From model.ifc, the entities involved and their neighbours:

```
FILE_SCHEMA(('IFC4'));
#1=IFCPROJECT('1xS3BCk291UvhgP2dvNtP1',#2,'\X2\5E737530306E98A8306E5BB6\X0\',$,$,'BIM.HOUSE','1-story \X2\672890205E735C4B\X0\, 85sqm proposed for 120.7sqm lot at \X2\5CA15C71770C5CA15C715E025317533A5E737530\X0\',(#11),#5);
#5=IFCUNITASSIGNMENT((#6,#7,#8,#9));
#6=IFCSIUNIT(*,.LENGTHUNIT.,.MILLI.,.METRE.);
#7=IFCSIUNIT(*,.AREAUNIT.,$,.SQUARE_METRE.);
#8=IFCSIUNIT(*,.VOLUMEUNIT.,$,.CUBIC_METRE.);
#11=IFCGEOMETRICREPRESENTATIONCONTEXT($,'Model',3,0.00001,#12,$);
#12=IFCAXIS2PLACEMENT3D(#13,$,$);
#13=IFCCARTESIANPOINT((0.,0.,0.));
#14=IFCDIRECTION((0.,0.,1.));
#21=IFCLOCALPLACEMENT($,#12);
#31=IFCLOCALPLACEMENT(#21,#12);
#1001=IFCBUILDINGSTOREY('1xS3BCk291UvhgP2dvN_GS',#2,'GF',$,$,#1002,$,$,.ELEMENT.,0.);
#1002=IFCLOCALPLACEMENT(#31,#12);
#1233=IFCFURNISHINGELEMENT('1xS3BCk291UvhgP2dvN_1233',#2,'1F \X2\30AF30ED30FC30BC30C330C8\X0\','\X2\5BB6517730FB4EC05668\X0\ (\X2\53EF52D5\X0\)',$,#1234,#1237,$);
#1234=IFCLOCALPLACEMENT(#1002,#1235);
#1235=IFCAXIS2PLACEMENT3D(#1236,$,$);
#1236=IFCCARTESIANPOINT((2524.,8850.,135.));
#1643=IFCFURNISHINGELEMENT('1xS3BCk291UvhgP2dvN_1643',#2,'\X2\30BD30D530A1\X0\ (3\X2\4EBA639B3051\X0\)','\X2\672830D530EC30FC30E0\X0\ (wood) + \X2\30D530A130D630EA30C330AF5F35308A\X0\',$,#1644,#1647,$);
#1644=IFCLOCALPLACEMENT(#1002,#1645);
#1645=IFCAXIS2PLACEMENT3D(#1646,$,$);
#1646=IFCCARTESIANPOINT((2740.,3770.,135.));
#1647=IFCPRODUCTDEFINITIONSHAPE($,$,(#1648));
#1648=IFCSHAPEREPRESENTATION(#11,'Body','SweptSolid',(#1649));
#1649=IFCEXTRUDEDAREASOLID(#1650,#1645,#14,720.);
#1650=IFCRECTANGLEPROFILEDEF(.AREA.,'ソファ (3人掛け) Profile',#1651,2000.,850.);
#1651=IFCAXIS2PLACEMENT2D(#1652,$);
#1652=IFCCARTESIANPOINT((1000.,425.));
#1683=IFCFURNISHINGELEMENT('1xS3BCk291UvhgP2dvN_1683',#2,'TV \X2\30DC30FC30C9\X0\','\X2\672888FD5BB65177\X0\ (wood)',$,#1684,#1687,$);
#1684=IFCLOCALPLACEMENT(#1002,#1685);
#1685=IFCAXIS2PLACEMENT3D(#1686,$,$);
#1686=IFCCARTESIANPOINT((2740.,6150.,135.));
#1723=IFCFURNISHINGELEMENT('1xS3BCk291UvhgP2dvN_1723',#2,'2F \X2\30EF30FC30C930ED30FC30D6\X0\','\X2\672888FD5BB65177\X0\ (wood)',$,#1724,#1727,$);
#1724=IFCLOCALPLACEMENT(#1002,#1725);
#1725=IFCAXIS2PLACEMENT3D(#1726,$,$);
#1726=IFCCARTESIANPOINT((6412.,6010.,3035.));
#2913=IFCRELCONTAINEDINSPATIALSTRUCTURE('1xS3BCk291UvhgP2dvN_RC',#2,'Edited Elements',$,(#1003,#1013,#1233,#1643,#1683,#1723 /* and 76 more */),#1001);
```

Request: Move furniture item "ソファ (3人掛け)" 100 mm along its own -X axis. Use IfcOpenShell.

```python
import ifcopenshell
import ifcopenshell.api.geometry
import ifcopenshell.util.placement

model = ifcopenshell.open("model.ifc")

item = model.by_guid("1xS3BCk291UvhgP2dvN_1643")
matrix = ifcopenshell.util.placement.get_local_placement(item.ObjectPlacement)
matrix[:3, 3] -= matrix[:3, 0] * 100.0
ifcopenshell.api.geometry.edit_object_placement(model, product=item, matrix=matrix, is_si=False)

print(ifcopenshell.util.placement.get_local_placement(item.ObjectPlacement).round(3) + 0.0)

model.write("model_updated.ifc")
```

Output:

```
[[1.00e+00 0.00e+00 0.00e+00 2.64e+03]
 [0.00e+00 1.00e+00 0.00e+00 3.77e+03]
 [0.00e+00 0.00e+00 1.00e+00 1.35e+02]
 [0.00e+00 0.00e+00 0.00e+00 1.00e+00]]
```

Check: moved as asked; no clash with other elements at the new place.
